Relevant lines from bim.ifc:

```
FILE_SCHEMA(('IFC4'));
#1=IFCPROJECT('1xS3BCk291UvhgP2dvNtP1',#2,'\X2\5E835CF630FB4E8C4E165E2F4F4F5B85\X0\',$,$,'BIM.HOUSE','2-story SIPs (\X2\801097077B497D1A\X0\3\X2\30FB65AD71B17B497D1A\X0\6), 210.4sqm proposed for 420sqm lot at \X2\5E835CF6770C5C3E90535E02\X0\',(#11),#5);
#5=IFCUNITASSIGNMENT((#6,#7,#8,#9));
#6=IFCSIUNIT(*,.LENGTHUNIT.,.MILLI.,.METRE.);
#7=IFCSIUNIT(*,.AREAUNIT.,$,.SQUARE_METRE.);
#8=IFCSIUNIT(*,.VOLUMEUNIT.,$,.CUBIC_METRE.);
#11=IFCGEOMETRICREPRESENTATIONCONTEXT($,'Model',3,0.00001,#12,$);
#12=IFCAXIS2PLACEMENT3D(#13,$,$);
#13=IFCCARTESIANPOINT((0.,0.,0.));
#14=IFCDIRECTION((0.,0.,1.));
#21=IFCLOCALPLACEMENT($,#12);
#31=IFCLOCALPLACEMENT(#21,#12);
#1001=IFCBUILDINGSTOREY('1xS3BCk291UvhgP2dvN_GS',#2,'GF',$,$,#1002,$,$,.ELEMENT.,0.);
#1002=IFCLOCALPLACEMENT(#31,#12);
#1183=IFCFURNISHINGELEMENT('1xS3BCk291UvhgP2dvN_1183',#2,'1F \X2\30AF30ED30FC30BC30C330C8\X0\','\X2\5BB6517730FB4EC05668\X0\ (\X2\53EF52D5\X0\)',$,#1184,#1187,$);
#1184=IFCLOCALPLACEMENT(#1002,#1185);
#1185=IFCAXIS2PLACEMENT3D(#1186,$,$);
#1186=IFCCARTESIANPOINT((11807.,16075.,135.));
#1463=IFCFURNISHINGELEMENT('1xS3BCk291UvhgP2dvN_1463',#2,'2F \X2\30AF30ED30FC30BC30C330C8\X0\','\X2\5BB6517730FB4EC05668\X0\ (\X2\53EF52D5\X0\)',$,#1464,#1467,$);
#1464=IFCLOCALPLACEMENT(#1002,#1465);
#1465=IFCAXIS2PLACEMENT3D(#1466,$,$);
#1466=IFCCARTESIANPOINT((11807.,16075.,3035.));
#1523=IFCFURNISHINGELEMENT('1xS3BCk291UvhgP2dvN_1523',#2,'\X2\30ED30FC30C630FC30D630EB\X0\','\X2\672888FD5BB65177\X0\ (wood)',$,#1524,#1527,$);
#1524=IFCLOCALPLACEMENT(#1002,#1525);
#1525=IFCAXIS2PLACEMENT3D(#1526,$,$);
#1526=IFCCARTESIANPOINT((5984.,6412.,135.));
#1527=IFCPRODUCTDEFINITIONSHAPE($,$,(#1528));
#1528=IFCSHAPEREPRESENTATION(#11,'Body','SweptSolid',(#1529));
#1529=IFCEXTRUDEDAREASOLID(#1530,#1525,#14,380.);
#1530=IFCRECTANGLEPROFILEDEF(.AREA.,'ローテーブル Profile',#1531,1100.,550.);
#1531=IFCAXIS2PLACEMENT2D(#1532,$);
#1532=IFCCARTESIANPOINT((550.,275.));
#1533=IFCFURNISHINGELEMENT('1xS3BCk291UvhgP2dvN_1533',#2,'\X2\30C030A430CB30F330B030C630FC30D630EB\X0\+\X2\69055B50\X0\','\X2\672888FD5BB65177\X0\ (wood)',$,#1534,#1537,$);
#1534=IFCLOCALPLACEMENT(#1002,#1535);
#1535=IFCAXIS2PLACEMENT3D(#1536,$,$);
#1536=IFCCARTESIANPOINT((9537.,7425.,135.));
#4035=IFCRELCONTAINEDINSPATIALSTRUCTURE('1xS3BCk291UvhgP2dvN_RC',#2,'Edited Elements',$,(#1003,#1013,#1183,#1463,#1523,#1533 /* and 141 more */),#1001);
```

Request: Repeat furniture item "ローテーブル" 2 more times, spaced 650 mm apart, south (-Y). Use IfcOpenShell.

```python
import numpy as np
import ifcopenshell
import ifcopenshell.api.geometry
import ifcopenshell.api.root
import ifcopenshell.util.element
import ifcopenshell.util.placement
import ifcopenshell.util.unit

model = ifcopenshell.open("bim.ifc")
unit_scale = ifcopenshell.util.unit.calculate_unit_scale(model)


def reuse_history(source, copy):
    """copy_class also copies each property set's owner history, people and application; keep the originals."""
    for rel in copy.IsDefinedBy:
        if rel.is_a("IfcRelDefinesByProperties") and (history := rel.RelatingPropertyDefinition.OwnerHistory):
            rel.RelatingPropertyDefinition.OwnerHistory = source.OwnerHistory
            ifcopenshell.util.element.remove_deep2(model, history)


source = model.by_guid("1xS3BCk291UvhgP2dvN_1523")
base = ifcopenshell.util.placement.get_local_placement(source.ObjectPlacement)
step = np.array([0.0, -1.0, 0.0]) * 0.65 / unit_scale

for i in range(1, 3):
    copy = ifcopenshell.api.root.copy_class(model, product=source)
    copy.Representation = ifcopenshell.util.element.copy_deep(
        model, source.Representation, exclude=["IfcGeometricRepresentationContext", "IfcRepresentationMap"]
    )
    reuse_history(source, copy)
    matrix = base.copy()
    matrix[:3, 3] += i * step
    print("added at", matrix[:3, 3].round(3) + 0.0)
    ifcopenshell.api.geometry.edit_object_placement(model, product=copy, matrix=matrix, is_si=False)

model.write("bim_updated.ifc")
```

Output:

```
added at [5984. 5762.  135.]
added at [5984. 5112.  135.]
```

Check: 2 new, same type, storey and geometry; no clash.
